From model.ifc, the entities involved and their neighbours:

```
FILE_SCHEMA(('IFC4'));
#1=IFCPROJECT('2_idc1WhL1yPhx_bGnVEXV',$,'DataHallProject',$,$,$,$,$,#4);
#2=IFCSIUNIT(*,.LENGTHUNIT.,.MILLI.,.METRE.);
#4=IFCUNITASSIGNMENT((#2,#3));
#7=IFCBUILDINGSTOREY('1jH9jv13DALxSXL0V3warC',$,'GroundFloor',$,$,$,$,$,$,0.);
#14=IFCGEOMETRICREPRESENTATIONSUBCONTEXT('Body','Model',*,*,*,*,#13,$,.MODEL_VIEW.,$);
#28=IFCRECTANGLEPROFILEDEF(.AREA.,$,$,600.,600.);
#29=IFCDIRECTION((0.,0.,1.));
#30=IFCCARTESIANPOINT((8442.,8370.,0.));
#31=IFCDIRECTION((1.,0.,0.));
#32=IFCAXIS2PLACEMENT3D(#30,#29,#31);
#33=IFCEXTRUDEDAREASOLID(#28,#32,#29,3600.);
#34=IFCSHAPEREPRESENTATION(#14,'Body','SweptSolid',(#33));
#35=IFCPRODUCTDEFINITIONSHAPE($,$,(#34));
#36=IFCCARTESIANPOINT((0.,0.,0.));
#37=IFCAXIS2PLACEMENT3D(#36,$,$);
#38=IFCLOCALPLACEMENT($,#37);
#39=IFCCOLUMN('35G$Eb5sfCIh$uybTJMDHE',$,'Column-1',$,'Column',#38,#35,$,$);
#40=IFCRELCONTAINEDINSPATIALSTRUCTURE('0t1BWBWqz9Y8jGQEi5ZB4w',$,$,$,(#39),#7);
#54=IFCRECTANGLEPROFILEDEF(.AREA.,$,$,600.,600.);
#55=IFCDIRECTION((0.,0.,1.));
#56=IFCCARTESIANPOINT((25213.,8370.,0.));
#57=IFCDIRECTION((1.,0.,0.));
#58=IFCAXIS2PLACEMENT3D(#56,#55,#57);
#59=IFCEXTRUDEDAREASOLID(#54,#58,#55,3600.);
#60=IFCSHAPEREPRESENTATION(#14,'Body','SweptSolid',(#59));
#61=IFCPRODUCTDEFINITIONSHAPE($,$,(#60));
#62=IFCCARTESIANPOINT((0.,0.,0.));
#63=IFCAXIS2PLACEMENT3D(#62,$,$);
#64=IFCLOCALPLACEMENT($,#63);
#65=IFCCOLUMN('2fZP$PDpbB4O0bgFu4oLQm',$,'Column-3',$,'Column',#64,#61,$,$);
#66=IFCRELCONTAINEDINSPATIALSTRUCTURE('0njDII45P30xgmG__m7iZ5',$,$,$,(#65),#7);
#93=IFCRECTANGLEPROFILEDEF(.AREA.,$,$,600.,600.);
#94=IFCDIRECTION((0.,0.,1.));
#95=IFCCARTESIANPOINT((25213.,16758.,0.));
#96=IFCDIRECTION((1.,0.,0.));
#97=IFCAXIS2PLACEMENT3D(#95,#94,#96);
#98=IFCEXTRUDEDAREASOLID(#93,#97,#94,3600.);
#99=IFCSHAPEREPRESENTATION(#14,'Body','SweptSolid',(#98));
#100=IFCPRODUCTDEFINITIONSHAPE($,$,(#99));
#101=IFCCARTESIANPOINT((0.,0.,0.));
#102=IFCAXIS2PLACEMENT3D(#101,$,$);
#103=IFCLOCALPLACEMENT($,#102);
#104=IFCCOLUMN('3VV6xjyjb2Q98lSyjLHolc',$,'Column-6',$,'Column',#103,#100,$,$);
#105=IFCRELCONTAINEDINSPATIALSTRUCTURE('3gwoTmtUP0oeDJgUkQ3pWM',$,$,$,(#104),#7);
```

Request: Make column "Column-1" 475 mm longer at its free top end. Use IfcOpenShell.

```python
import ifcopenshell
import ifcopenshell.util.representation

model = ifcopenshell.open("model.ifc")

member = model.by_id(39)
change = 475.0

# The extrusion runs towards the end named, so only its depth changes.
body = ifcopenshell.util.representation.get_representation(member, "Model", "Body")
solid = body.Items[0]
old_length = solid.Depth
solid.Depth += change

print(f"length {old_length:g} -> {solid.Depth:g}")

model.write("model_rev.ifc")
```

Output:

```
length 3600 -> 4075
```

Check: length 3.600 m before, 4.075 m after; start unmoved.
